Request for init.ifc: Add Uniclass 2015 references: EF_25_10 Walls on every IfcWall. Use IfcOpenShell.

First a look at what the model holds.

```python
import ifcopenshell

model = ifcopenshell.open("init.ifc")
print(model.schema)
print("classifications:", [c.Name for c in model.by_type("IfcClassification")])
for ifc_class in ("IfcDoor", "IfcRoof", "IfcStair", "IfcWall", "IfcWindow"):
    print(ifc_class, len(model.by_type(ifc_class)))
```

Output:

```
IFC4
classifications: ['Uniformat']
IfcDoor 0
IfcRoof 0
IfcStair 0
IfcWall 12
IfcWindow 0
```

```python
import ifcopenshell
import ifcopenshell.api.classification

model = ifcopenshell.open("init.ifc")

system = ifcopenshell.api.classification.add_classification(model, classification="Uniclass 2015")

codes = {
    "IfcWall": ("EF_25_10", "Walls"),
}
for ifc_class, (code, name) in codes.items():
    products = model.by_type(ifc_class)
    ifcopenshell.api.classification.add_reference(
        model, products=products, classification=system, identification=code, name=name
    )
    print(code, len(products))

model.write("init-out.ifc")
```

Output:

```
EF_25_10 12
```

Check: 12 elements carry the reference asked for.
